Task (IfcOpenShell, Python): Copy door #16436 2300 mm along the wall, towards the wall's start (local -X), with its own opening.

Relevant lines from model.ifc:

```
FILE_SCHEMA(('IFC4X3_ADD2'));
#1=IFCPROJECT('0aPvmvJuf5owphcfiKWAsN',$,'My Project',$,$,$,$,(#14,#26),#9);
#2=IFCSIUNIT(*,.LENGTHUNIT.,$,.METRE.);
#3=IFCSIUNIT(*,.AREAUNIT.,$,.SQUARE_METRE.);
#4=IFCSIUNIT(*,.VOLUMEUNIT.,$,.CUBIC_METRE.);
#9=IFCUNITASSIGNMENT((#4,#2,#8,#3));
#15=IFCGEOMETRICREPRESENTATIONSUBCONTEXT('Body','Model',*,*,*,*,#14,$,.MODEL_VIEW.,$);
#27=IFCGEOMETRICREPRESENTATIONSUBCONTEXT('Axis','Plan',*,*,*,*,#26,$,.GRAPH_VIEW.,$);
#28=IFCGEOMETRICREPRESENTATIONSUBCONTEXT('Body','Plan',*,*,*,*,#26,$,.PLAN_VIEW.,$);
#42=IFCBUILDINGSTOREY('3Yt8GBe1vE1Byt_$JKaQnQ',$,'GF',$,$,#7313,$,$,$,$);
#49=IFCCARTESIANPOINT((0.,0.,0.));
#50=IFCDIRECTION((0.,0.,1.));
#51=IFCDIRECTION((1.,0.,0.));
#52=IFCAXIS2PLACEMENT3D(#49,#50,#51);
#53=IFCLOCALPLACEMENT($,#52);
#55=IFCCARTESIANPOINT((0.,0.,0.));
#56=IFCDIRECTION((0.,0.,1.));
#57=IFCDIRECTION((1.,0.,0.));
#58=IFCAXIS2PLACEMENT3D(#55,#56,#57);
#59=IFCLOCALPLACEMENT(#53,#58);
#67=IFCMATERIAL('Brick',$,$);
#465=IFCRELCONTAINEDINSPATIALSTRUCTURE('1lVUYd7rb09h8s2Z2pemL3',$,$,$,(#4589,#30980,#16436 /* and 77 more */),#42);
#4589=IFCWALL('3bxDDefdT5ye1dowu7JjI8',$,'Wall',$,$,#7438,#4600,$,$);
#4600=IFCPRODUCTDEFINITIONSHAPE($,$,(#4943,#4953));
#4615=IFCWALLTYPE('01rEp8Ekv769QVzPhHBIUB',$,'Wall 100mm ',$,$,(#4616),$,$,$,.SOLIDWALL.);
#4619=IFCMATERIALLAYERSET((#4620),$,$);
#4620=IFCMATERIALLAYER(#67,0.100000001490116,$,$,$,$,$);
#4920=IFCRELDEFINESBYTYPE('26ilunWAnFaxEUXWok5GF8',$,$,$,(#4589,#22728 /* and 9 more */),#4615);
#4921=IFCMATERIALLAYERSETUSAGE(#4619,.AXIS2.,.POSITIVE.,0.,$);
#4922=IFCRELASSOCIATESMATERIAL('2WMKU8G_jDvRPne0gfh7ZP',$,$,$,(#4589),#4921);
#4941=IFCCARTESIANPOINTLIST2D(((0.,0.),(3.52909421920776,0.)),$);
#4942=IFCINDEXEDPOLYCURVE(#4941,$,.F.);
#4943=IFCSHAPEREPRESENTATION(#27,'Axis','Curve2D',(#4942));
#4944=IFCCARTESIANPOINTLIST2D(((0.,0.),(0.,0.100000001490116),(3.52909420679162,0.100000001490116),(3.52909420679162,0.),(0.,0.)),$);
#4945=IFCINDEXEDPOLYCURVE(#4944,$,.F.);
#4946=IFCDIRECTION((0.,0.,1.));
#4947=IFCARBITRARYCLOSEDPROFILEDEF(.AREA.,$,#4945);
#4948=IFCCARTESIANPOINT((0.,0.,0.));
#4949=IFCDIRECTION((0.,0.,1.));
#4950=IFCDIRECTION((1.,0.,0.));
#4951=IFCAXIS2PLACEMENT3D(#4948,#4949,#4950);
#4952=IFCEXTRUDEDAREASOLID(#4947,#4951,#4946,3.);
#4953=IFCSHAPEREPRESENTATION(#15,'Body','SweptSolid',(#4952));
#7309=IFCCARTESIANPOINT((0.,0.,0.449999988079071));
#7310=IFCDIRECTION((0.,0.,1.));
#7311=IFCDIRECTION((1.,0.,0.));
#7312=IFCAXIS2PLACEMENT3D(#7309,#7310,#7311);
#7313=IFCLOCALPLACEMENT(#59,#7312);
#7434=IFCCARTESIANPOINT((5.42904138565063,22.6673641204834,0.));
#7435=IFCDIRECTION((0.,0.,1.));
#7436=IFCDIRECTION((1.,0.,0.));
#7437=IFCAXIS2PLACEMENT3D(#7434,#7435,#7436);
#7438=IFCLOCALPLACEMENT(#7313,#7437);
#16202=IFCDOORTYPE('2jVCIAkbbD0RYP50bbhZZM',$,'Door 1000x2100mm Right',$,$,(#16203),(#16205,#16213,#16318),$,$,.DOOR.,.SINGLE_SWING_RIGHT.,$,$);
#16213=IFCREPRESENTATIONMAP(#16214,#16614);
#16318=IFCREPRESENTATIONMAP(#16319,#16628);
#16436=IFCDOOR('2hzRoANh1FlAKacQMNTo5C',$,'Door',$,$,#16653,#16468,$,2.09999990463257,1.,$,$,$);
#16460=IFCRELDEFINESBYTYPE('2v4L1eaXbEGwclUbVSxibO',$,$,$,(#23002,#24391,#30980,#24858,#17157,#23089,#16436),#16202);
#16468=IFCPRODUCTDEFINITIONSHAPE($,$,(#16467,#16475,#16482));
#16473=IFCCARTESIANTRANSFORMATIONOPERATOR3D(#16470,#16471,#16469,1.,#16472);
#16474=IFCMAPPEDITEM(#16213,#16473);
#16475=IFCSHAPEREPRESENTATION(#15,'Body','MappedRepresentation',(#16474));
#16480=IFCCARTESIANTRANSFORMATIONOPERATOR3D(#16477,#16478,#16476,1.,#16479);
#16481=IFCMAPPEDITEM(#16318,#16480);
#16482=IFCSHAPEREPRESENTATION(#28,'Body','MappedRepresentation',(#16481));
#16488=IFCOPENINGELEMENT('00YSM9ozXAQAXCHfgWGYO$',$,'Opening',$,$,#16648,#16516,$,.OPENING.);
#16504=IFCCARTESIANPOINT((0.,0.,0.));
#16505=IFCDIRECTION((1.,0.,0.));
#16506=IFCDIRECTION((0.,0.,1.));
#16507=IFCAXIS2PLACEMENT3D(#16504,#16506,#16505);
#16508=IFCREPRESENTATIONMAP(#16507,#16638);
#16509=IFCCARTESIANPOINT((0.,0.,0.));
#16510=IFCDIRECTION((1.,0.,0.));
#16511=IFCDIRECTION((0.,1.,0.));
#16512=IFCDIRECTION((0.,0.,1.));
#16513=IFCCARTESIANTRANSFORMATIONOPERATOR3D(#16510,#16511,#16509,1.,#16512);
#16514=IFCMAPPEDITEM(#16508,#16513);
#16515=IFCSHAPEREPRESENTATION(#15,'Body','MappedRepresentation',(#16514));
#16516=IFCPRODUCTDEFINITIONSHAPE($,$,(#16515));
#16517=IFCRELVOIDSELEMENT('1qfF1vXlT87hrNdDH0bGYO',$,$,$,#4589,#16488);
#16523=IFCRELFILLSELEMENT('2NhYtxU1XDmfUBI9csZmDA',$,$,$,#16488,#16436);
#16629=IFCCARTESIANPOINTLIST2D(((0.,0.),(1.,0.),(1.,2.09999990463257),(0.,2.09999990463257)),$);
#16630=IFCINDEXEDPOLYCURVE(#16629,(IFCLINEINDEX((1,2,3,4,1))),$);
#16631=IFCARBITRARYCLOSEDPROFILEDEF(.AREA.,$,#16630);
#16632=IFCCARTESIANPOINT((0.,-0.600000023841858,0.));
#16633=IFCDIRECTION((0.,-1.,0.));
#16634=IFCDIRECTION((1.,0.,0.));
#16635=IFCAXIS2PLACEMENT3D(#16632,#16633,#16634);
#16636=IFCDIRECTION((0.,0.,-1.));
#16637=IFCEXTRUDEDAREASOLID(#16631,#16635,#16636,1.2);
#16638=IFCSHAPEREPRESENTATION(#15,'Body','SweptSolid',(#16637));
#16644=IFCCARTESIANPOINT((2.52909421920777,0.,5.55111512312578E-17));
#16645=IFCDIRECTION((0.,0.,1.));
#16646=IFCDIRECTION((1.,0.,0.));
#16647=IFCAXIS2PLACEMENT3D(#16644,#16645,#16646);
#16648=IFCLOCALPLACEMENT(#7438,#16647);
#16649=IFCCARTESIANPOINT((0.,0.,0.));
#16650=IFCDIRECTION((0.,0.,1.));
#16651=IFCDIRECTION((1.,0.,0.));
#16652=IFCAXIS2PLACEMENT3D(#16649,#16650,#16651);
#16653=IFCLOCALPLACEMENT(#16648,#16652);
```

```python
import ifcopenshell
import ifcopenshell.api.feature
import ifcopenshell.api.geometry
import ifcopenshell.api.root
import ifcopenshell.geom
import ifcopenshell.util.element
import ifcopenshell.util.placement
import ifcopenshell.util.shape

model = ifcopenshell.open("model.ifc")
settings = ifcopenshell.geom.settings()


def volume(element):
    """Net volume in cubic metres, openings subtracted."""
    shape = ifcopenshell.geom.create_shape(settings, element)
    return ifcopenshell.util.shape.get_volume(shape.geometry)


door = model.by_guid("2hzRoANh1FlAKacQMNTo5C")
opening = door.FillsVoids[0].RelatingOpeningElement
wall = opening.VoidsElements[0].RelatingBuildingElement
before = volume(wall)
shift = ifcopenshell.util.placement.get_local_placement(wall.ObjectPlacement)[:3, 0] * -2.3

# copy_class copies the void relationship, type, container and properties, but no geometry.
new_opening = ifcopenshell.api.root.copy_class(model, product=opening)
new_opening.Representation = ifcopenshell.util.element.copy_deep(
    model, opening.Representation, exclude=["IfcGeometricRepresentationContext", "IfcRepresentationMap"]
)
new_door = ifcopenshell.api.root.copy_class(model, product=door)
new_door.Representation = ifcopenshell.util.element.copy_deep(
    model, door.Representation, exclude=["IfcGeometricRepresentationContext", "IfcRepresentationMap"]
)
ifcopenshell.api.feature.add_filling(model, opening=new_opening, element=new_door)

for old, new in ((opening, new_opening), (door, new_door)):
    matrix = ifcopenshell.util.placement.get_local_placement(old.ObjectPlacement)
    matrix[:3, 3] += shift
    ifcopenshell.api.geometry.edit_object_placement(model, product=new, matrix=matrix, is_si=False)

after = volume(wall)

print(f"wall volume {before:.3f} -> {after:.3f} m3")

model.write("model_updated.ifc")
```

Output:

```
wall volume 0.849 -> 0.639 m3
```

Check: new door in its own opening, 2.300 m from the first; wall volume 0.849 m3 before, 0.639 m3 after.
